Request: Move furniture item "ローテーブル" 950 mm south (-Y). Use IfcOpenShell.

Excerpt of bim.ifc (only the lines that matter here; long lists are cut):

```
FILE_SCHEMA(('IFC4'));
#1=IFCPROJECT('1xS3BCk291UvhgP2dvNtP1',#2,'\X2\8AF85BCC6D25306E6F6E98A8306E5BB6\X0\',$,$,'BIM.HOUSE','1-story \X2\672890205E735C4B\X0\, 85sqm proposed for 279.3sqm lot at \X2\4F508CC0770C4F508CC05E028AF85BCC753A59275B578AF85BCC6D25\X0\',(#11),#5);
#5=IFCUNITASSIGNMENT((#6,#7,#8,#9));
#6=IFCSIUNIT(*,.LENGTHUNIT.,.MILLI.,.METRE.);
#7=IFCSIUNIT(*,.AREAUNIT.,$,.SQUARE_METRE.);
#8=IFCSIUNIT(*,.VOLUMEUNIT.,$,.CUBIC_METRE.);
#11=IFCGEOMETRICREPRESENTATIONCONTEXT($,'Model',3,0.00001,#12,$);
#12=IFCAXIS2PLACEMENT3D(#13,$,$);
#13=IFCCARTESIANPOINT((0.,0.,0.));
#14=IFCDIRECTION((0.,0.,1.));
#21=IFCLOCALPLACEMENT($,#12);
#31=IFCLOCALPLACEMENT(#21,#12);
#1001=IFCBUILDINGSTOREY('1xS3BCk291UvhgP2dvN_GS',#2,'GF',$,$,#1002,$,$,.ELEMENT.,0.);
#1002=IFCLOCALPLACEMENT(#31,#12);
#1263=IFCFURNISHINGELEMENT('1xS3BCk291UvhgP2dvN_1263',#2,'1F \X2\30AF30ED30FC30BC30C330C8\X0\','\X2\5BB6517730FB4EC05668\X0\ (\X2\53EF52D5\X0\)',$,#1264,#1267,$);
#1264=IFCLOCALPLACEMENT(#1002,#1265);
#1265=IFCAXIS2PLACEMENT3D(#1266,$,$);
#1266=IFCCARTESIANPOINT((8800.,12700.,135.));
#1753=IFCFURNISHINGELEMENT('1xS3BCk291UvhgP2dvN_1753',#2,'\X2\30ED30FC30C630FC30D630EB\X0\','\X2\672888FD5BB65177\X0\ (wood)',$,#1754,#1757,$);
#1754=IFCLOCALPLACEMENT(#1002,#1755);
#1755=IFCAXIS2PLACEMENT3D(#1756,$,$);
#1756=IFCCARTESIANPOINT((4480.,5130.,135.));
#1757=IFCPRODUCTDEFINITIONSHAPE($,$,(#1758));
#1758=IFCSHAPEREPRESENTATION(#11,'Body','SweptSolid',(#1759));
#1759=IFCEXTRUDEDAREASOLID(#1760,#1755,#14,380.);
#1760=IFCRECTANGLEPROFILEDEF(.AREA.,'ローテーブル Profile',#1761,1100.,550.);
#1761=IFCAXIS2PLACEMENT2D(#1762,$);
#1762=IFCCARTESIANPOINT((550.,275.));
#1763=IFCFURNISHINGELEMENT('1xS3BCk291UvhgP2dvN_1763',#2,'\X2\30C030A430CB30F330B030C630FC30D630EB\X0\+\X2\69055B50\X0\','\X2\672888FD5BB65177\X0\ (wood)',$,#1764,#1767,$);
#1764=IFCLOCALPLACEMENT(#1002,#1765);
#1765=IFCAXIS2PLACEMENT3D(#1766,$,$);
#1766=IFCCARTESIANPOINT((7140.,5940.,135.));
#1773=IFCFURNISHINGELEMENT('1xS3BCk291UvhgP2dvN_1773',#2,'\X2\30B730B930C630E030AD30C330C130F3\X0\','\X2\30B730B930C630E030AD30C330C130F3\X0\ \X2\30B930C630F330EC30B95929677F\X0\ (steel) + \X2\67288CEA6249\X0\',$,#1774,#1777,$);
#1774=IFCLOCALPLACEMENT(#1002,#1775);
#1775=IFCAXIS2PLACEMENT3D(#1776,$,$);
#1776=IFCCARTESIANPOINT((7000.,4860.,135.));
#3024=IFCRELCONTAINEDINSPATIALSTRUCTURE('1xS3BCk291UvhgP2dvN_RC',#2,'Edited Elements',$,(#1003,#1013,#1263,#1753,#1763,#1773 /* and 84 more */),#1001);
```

```python
import ifcopenshell
import ifcopenshell.api.geometry
import ifcopenshell.util.placement
import ifcopenshell.util.unit

model = ifcopenshell.open("bim.ifc")
unit_scale = ifcopenshell.util.unit.calculate_unit_scale(model)

item = model.by_guid("1xS3BCk291UvhgP2dvN_1753")
matrix = ifcopenshell.util.placement.get_local_placement(item.ObjectPlacement)
matrix[1, 3] -= 0.95 / unit_scale
ifcopenshell.api.geometry.edit_object_placement(model, product=item, matrix=matrix, is_si=False)

print(ifcopenshell.util.placement.get_local_placement(item.ObjectPlacement).round(3) + 0.0)

model.write("bim_edited.ifc")
```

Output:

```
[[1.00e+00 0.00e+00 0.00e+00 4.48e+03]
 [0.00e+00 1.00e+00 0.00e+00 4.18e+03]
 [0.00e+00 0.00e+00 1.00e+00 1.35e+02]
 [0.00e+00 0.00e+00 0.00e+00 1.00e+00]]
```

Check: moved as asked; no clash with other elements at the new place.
